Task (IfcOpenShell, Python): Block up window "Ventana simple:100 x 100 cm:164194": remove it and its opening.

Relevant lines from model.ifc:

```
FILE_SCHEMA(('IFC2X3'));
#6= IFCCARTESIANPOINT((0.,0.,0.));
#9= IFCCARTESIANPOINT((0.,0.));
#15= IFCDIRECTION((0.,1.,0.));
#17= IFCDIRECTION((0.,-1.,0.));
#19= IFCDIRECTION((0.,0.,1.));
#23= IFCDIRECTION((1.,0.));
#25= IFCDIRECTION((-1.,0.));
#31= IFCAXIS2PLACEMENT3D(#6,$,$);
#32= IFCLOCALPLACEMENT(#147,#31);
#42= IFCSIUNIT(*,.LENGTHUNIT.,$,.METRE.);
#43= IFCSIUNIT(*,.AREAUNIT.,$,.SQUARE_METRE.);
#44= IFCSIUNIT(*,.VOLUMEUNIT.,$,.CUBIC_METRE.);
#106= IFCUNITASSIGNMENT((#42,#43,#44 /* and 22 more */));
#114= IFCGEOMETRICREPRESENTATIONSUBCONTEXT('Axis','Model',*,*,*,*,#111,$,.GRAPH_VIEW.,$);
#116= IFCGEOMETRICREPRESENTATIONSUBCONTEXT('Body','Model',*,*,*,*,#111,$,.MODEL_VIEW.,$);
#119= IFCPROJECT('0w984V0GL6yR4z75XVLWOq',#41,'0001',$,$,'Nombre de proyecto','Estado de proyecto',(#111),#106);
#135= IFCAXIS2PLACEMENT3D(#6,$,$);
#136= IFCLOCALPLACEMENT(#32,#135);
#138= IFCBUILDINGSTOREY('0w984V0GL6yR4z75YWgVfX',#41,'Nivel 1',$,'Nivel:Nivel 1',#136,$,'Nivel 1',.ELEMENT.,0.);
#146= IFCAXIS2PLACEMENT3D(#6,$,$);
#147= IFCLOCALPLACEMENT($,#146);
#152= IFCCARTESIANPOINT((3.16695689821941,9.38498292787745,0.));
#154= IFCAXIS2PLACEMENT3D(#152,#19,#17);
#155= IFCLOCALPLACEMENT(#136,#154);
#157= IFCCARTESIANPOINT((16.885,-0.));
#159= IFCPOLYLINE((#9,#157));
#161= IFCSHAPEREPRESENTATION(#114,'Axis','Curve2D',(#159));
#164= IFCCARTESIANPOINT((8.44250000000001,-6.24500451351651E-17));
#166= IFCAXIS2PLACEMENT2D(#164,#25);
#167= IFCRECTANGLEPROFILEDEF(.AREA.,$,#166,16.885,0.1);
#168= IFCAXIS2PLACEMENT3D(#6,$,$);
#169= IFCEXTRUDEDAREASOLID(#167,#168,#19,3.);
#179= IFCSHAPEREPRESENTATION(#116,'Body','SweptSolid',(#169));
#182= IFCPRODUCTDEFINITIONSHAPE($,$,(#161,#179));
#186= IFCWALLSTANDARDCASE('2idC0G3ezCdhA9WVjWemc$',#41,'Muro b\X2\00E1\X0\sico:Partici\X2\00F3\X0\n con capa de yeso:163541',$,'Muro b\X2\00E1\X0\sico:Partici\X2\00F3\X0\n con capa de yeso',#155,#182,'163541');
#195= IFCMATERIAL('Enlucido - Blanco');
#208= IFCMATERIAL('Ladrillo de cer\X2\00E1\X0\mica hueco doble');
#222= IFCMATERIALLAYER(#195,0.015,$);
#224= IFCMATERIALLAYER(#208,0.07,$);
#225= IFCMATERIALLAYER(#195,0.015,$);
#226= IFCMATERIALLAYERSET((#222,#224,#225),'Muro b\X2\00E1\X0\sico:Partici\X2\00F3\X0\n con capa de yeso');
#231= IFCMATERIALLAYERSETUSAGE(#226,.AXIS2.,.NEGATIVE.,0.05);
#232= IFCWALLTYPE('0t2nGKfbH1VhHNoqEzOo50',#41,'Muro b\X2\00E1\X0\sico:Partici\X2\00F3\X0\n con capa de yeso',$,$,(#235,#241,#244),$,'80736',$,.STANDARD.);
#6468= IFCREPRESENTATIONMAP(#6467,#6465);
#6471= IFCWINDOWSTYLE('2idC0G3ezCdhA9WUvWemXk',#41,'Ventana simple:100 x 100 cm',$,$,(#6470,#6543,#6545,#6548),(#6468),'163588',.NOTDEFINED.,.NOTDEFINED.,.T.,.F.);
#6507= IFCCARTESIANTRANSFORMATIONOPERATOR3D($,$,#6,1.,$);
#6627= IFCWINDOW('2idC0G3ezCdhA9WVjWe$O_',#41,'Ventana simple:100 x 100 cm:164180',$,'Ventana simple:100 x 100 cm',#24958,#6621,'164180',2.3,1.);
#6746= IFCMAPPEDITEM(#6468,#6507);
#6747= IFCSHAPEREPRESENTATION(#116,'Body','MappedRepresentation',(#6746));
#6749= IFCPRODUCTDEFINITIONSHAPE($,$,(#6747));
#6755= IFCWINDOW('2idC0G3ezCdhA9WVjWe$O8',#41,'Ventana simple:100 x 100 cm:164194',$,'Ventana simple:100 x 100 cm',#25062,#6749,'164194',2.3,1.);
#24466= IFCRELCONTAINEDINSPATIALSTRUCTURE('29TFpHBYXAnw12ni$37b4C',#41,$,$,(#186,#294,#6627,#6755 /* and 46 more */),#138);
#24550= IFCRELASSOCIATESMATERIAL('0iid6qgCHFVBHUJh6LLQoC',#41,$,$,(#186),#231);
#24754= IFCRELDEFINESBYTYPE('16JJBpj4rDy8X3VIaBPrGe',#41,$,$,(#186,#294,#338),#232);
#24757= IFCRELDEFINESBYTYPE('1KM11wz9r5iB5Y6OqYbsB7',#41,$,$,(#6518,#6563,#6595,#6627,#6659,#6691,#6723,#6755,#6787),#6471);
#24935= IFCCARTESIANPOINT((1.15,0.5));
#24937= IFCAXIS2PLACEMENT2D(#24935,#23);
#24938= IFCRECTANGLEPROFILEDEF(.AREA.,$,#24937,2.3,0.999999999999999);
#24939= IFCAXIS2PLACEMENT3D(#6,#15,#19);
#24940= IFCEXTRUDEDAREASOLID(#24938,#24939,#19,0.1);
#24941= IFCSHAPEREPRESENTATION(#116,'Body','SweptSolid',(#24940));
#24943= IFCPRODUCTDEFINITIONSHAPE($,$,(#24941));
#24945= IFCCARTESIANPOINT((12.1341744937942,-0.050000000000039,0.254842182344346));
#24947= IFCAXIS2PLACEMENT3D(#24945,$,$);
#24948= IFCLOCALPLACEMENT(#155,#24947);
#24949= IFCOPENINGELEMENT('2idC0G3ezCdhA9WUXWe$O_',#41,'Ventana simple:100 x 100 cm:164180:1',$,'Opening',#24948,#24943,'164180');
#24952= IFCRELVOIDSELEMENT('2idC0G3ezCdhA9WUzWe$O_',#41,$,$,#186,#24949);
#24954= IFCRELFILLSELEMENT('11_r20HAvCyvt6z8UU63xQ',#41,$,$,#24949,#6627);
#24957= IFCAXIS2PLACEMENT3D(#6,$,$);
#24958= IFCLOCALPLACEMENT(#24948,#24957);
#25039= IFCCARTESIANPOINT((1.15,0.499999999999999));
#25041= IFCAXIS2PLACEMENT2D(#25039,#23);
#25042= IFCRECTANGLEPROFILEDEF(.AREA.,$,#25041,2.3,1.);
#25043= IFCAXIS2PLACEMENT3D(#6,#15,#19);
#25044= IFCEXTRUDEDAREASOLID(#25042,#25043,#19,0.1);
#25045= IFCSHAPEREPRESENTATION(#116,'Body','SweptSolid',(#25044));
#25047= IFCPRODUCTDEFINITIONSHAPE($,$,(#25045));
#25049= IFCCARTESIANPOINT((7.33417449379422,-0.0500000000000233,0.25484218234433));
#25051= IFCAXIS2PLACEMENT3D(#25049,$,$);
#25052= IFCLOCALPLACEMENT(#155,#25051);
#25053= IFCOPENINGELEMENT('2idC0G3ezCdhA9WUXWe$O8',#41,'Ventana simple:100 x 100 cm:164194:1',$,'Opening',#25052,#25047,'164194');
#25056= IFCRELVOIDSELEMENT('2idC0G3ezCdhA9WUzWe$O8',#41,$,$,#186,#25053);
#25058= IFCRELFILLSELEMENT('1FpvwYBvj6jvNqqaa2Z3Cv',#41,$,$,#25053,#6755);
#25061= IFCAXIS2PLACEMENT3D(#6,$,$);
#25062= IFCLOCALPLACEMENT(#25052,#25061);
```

```python
import ifcopenshell
import ifcopenshell.api.feature
import ifcopenshell.api.root
import ifcopenshell.geom
import ifcopenshell.util.shape

model = ifcopenshell.open("model.ifc")
settings = ifcopenshell.geom.settings()


def volume(element):
    """Net volume in cubic metres, openings subtracted."""
    shape = ifcopenshell.geom.create_shape(settings, element)
    return ifcopenshell.util.shape.get_volume(shape.geometry)


window = model.by_id(6755)
opening = window.FillsVoids[0].RelatingOpeningElement
wall = opening.VoidsElements[0].RelatingBuildingElement
before = volume(wall)

ifcopenshell.api.root.remove_product(model, product=window)
ifcopenshell.api.feature.remove_feature(model, feature=opening)

after = volume(wall)

print(f"wall volume {before:.3f} -> {after:.3f} m3")

model.write("model-out.ifc")
```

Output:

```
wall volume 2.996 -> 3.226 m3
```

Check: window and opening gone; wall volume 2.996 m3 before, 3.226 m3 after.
